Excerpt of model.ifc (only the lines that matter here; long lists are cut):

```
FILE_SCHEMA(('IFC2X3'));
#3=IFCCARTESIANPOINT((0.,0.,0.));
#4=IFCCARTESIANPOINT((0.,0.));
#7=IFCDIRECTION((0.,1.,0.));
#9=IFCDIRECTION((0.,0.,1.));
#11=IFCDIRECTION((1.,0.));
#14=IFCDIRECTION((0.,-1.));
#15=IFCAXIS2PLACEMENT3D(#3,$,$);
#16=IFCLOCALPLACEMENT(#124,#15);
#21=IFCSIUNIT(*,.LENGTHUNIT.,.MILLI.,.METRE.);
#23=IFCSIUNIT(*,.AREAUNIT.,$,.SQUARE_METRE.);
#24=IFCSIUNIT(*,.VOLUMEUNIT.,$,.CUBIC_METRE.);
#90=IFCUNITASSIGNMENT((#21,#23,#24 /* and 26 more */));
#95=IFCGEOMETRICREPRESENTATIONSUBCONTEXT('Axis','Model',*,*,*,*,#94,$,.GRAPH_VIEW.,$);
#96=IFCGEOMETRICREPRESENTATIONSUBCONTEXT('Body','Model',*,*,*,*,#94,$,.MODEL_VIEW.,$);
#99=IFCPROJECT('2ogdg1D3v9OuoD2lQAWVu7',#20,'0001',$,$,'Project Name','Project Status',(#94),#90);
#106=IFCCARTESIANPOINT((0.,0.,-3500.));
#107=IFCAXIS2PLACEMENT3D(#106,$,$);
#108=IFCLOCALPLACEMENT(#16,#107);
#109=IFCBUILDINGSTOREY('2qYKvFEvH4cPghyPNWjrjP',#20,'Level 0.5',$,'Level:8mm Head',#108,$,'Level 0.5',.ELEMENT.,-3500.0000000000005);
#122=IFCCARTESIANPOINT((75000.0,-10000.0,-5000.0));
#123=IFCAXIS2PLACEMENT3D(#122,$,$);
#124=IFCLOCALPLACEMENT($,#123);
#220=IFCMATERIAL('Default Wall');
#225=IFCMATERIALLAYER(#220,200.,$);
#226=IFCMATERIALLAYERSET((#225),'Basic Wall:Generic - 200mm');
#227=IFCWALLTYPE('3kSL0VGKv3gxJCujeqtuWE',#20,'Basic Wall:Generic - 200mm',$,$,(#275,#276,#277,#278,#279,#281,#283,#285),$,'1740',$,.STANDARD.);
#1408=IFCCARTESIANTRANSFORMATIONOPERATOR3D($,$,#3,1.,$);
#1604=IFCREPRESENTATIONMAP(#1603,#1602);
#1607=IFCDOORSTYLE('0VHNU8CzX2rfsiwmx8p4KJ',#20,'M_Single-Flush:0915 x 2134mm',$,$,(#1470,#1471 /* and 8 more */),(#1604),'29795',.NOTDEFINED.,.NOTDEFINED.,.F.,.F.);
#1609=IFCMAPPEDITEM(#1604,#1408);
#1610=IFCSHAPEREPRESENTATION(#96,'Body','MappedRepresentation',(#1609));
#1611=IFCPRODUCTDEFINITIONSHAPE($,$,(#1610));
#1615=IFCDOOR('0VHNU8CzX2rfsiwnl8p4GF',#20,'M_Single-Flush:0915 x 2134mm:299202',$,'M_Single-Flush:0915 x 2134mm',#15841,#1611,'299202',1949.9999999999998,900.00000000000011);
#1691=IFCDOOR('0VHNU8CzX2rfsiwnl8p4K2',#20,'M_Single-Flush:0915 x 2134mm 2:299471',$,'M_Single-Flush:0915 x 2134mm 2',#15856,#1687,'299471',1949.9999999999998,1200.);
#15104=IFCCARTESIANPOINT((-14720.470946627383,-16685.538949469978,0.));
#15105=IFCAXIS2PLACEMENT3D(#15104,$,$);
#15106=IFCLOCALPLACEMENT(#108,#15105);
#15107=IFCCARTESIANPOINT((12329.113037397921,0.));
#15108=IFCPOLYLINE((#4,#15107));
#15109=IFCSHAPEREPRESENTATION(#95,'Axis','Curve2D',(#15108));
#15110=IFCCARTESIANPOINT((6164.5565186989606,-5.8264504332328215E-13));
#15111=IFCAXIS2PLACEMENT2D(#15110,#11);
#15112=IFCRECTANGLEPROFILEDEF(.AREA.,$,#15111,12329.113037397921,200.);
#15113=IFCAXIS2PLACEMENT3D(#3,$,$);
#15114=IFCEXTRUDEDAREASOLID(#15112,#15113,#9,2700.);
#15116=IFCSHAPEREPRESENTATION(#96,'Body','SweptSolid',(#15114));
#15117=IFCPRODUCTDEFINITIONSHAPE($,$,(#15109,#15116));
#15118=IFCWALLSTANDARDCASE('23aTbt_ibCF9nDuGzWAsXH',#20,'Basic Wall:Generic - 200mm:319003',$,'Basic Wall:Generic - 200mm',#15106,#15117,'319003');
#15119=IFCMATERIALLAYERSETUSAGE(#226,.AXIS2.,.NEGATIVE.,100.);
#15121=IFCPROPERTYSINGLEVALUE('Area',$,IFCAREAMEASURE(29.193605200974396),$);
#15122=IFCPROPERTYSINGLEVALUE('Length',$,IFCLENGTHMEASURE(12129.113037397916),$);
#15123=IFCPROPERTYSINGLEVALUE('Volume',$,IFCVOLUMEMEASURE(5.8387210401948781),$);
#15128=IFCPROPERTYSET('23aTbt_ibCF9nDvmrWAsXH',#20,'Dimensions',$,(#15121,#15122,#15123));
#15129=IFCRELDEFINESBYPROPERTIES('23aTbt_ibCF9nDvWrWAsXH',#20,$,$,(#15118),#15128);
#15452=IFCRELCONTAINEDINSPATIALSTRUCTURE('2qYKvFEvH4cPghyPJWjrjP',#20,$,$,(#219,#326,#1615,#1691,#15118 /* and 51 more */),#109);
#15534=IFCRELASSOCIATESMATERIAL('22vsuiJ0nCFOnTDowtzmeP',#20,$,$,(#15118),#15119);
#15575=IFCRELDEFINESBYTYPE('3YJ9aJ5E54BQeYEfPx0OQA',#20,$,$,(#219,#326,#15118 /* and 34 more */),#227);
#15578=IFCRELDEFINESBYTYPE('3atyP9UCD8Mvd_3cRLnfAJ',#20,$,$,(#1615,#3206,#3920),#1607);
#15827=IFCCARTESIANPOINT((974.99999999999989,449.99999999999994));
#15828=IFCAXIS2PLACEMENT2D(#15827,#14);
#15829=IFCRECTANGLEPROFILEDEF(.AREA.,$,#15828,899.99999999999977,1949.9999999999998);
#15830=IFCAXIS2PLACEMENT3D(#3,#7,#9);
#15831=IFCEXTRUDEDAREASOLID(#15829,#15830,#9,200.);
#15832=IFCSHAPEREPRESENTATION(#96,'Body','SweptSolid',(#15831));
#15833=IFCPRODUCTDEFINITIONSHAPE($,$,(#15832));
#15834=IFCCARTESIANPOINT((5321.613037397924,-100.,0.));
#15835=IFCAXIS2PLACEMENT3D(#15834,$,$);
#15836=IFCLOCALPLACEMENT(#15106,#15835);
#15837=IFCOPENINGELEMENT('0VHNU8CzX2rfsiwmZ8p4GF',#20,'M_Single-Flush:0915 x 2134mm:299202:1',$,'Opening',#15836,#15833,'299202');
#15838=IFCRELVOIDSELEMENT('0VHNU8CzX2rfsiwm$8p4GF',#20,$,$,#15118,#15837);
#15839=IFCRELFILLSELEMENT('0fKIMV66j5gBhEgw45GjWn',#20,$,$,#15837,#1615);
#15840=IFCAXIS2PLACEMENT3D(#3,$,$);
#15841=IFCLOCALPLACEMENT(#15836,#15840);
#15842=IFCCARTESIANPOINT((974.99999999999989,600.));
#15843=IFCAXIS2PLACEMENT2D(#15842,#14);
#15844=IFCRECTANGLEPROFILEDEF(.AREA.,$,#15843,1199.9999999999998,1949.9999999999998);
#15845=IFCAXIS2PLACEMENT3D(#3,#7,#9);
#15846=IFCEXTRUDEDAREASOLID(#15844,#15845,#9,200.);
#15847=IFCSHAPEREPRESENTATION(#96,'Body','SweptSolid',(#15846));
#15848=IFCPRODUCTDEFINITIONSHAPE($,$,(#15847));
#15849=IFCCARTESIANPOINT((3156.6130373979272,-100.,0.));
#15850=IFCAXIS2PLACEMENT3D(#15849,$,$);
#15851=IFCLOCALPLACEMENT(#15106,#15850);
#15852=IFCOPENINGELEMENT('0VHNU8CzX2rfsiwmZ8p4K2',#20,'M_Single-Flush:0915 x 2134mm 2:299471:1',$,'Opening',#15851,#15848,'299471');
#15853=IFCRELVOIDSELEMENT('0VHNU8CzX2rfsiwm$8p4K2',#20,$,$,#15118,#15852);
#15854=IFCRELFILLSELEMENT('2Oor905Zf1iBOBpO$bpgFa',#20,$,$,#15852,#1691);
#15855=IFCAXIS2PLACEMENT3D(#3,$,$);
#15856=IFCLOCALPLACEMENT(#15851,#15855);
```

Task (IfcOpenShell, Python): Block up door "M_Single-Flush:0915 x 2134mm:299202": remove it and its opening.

```python
import ifcopenshell
import ifcopenshell.api.feature
import ifcopenshell.api.pset
import ifcopenshell.api.root
import ifcopenshell.geom
import ifcopenshell.util.element
import ifcopenshell.util.shape
import ifcopenshell.util.unit

model = ifcopenshell.open("model.ifc")
area_scale = ifcopenshell.util.unit.calculate_unit_scale(model, "AREAUNIT")
volume_scale = ifcopenshell.util.unit.calculate_unit_scale(model, "VOLUMEUNIT")
settings = ifcopenshell.geom.settings()


def volume(element):
    """Net volume in cubic metres, openings subtracted."""
    shape = ifcopenshell.geom.create_shape(settings, element)
    return ifcopenshell.util.shape.get_volume(shape.geometry)


door = model.by_id(1615)
opening = door.FillsVoids[0].RelatingOpeningElement
wall = opening.VoidsElements[0].RelatingBuildingElement
before = volume(wall)

ifcopenshell.api.root.remove_product(model, product=door)
ifcopenshell.api.feature.remove_feature(model, feature=opening)

after = volume(wall)
thickness = 0.2  # wall thickness in metres

# Update the wall's stored quantities.
pset = model.by_id(ifcopenshell.util.element.get_pset(wall, "Dimensions", should_inherit=False)["id"])
ifcopenshell.api.pset.edit_pset(model, pset=pset, properties={
    "Area": model.create_entity("IfcAreaMeasure", after / thickness / area_scale),
    "Volume": model.create_entity("IfcVolumeMeasure", after / volume_scale),
})

print(f"wall volume {before:.3f} -> {after:.3f} m3")

model.write("model_rev.ifc")
```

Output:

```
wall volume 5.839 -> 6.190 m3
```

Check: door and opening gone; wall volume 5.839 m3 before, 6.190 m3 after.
